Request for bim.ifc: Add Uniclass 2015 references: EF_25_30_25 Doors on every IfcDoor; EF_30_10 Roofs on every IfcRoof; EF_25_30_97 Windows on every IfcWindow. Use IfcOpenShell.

First a look at what the model holds.

```python
import ifcopenshell

model = ifcopenshell.open("bim.ifc")
print(model.schema)
print("classifications:", [c.Name for c in model.by_type("IfcClassification")])
for ifc_class in ("IfcDoor", "IfcRoof", "IfcStair", "IfcWall", "IfcWindow"):
    print(ifc_class, len(model.by_type(ifc_class)))
```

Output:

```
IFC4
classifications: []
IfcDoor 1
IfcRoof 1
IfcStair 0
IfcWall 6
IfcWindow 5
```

```python
import ifcopenshell
import ifcopenshell.api.classification

model = ifcopenshell.open("bim.ifc")

system = ifcopenshell.api.classification.add_classification(model, classification="Uniclass 2015")

codes = {
    "IfcDoor": ("EF_25_30_25", "Doors"),
    "IfcRoof": ("EF_30_10", "Roofs"),
    "IfcWindow": ("EF_25_30_97", "Windows"),
}
for ifc_class, (code, name) in codes.items():
    products = model.by_type(ifc_class)
    ifcopenshell.api.classification.add_reference(
        model, products=products, classification=system, identification=code, name=name
    )
    print(code, len(products))

model.write("bim_updated.ifc")
```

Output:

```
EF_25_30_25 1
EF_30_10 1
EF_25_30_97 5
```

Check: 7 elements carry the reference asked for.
